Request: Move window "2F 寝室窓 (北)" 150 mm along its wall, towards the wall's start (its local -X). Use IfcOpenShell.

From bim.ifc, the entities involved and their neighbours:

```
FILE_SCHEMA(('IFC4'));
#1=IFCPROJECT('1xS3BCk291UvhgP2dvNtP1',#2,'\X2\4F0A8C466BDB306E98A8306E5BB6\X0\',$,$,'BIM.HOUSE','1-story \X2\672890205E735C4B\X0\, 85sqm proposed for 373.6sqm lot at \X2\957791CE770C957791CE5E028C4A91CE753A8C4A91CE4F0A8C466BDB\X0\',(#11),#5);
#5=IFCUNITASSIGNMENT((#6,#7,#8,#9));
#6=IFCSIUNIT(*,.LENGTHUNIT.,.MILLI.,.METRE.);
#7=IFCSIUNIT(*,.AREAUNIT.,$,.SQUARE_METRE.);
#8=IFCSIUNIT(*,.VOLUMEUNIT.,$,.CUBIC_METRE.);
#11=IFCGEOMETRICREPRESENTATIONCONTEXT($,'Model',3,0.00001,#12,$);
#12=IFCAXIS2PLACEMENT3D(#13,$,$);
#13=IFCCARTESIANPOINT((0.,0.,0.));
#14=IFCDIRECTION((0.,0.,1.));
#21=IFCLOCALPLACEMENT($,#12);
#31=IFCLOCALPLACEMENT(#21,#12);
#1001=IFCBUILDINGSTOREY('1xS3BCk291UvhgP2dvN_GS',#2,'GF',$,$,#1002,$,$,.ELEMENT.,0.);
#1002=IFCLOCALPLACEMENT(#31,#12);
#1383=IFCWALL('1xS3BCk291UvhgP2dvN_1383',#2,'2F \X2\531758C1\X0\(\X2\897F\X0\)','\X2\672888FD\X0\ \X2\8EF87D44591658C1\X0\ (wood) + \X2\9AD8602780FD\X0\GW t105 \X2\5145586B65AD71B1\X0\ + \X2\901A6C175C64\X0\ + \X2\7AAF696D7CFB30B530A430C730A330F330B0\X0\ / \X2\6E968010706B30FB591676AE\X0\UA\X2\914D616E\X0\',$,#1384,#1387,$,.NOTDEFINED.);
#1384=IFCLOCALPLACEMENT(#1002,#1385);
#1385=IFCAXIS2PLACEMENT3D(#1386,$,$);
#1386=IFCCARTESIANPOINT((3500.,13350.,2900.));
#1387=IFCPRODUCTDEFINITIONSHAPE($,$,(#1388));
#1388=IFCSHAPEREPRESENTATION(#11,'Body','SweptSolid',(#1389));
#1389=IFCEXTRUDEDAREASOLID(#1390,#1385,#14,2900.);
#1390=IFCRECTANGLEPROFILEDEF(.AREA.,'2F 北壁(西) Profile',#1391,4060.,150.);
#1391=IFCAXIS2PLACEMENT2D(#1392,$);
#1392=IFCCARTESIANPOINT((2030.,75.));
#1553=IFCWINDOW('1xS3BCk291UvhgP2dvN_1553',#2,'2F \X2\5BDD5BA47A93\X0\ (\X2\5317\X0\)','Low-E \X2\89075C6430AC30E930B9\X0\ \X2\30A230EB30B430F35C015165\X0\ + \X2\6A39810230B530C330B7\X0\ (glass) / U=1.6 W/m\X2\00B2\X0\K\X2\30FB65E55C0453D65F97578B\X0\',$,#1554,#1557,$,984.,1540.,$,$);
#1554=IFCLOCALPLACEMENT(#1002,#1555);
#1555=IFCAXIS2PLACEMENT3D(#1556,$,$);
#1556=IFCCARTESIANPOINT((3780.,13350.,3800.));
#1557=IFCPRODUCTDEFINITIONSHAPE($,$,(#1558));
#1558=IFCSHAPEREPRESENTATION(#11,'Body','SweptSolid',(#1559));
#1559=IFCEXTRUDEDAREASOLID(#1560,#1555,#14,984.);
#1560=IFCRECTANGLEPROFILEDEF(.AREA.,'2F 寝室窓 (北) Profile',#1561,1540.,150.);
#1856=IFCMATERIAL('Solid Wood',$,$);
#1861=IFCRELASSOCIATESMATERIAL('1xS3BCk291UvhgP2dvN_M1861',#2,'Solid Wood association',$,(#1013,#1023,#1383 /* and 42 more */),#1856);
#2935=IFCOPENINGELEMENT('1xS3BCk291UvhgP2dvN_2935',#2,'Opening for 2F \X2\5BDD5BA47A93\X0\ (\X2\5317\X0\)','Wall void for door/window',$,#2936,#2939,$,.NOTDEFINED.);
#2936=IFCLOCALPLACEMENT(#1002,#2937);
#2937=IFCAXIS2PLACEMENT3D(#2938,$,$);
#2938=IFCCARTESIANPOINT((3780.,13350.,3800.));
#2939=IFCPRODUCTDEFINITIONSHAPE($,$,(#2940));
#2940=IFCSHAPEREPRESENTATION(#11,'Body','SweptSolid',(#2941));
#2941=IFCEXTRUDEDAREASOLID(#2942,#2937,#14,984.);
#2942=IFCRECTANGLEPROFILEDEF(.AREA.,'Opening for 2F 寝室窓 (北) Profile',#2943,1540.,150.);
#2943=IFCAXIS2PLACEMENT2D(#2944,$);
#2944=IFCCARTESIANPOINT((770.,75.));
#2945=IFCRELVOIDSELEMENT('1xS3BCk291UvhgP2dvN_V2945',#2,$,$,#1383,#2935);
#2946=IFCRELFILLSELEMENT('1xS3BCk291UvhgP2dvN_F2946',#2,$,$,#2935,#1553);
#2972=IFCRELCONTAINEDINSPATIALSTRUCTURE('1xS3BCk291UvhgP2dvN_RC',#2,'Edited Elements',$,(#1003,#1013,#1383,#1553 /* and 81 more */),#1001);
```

```python
import ifcopenshell
import ifcopenshell.api.geometry
import ifcopenshell.util.placement
import ifcopenshell.util.unit

model = ifcopenshell.open("bim.ifc")
unit_scale = ifcopenshell.util.unit.calculate_unit_scale(model)

window = model.by_guid("1xS3BCk291UvhgP2dvN_1553")
opening = window.FillsVoids[0].RelatingOpeningElement
wall = opening.VoidsElements[0].RelatingBuildingElement

wall_matrix = ifcopenshell.util.placement.get_local_placement(wall.ObjectPlacement)
shift = wall_matrix[:3, 0] * -0.15 / unit_scale
before = ifcopenshell.util.placement.get_local_placement(window.ObjectPlacement)[:3, 3].copy()

# The window is not placed relative to its opening, so move both.
for product in (opening, window):
    matrix = ifcopenshell.util.placement.get_local_placement(product.ObjectPlacement)
    matrix[:3, 3] += shift
    ifcopenshell.api.geometry.edit_object_placement(model, product=product, matrix=matrix, is_si=False)

after = ifcopenshell.util.placement.get_local_placement(window.ObjectPlacement)[:3, 3]
print("window moved by", (after - before).round(3) + 0.0)

model.write("bim_v2.ifc")
```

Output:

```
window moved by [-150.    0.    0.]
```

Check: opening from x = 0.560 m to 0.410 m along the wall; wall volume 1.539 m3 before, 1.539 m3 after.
